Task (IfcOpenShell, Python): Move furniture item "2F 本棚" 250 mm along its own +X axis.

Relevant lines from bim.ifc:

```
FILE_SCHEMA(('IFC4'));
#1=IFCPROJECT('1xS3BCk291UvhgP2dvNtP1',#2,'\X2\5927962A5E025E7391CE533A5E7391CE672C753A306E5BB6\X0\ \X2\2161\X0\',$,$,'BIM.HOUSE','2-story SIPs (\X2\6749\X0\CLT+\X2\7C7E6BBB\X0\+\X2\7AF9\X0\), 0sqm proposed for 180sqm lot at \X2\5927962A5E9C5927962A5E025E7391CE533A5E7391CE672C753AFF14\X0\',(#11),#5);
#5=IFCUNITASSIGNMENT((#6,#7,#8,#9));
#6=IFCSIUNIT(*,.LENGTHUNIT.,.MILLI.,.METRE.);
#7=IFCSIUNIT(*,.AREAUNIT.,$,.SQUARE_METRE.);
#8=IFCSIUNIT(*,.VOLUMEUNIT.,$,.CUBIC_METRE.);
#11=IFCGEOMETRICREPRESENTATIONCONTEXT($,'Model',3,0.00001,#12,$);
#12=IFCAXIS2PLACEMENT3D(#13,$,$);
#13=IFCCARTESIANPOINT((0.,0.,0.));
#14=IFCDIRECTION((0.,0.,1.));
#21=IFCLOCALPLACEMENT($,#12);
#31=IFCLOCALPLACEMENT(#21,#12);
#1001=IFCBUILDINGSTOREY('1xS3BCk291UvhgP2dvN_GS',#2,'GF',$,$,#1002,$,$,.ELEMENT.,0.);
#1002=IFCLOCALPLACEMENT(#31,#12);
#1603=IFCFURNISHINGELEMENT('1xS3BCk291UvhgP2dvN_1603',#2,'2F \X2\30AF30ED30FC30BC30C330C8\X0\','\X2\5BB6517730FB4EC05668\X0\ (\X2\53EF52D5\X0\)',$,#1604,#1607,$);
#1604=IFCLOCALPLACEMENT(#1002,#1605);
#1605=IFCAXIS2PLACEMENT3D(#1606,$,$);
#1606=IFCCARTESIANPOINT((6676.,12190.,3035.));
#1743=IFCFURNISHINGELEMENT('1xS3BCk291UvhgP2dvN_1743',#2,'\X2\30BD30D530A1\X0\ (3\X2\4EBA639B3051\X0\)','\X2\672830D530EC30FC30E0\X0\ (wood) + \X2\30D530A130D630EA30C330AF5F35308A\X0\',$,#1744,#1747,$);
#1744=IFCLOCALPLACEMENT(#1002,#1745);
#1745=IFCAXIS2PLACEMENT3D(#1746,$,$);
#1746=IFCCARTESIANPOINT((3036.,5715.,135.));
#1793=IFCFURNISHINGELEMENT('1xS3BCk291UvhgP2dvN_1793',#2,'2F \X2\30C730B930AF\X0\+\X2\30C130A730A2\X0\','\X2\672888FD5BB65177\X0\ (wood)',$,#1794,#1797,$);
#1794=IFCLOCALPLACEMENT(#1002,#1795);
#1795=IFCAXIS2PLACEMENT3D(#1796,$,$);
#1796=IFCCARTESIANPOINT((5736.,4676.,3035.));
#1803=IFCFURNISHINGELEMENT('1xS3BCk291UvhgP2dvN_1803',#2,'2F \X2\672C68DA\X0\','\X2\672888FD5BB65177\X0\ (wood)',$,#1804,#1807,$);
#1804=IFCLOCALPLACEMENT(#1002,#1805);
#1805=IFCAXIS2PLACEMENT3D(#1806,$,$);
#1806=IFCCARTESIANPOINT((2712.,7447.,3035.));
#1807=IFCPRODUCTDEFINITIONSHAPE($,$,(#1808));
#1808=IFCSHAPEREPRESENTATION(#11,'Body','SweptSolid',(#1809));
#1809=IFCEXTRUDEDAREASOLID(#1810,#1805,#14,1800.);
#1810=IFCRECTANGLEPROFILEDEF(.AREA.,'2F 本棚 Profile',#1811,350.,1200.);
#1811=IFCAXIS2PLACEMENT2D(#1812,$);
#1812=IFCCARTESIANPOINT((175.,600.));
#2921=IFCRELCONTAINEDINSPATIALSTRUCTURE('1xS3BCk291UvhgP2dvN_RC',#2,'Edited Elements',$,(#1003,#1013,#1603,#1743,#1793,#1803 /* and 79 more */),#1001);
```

```python
import ifcopenshell
import ifcopenshell.api.geometry
import ifcopenshell.util.placement
import ifcopenshell.util.unit

model = ifcopenshell.open("bim.ifc")
unit_scale = ifcopenshell.util.unit.calculate_unit_scale(model)

item = model.by_guid("1xS3BCk291UvhgP2dvN_1803")
matrix = ifcopenshell.util.placement.get_local_placement(item.ObjectPlacement)
matrix[:3, 3] += matrix[:3, 0] * 0.25 / unit_scale
ifcopenshell.api.geometry.edit_object_placement(model, product=item, matrix=matrix, is_si=False)

print(ifcopenshell.util.placement.get_local_placement(item.ObjectPlacement).round(3) + 0.0)

model.write("bim-out.ifc")
```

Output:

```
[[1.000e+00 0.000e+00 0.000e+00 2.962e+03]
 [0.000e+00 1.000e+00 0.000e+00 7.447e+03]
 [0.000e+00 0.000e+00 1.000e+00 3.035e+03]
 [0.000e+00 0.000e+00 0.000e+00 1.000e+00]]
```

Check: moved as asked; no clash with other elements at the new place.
